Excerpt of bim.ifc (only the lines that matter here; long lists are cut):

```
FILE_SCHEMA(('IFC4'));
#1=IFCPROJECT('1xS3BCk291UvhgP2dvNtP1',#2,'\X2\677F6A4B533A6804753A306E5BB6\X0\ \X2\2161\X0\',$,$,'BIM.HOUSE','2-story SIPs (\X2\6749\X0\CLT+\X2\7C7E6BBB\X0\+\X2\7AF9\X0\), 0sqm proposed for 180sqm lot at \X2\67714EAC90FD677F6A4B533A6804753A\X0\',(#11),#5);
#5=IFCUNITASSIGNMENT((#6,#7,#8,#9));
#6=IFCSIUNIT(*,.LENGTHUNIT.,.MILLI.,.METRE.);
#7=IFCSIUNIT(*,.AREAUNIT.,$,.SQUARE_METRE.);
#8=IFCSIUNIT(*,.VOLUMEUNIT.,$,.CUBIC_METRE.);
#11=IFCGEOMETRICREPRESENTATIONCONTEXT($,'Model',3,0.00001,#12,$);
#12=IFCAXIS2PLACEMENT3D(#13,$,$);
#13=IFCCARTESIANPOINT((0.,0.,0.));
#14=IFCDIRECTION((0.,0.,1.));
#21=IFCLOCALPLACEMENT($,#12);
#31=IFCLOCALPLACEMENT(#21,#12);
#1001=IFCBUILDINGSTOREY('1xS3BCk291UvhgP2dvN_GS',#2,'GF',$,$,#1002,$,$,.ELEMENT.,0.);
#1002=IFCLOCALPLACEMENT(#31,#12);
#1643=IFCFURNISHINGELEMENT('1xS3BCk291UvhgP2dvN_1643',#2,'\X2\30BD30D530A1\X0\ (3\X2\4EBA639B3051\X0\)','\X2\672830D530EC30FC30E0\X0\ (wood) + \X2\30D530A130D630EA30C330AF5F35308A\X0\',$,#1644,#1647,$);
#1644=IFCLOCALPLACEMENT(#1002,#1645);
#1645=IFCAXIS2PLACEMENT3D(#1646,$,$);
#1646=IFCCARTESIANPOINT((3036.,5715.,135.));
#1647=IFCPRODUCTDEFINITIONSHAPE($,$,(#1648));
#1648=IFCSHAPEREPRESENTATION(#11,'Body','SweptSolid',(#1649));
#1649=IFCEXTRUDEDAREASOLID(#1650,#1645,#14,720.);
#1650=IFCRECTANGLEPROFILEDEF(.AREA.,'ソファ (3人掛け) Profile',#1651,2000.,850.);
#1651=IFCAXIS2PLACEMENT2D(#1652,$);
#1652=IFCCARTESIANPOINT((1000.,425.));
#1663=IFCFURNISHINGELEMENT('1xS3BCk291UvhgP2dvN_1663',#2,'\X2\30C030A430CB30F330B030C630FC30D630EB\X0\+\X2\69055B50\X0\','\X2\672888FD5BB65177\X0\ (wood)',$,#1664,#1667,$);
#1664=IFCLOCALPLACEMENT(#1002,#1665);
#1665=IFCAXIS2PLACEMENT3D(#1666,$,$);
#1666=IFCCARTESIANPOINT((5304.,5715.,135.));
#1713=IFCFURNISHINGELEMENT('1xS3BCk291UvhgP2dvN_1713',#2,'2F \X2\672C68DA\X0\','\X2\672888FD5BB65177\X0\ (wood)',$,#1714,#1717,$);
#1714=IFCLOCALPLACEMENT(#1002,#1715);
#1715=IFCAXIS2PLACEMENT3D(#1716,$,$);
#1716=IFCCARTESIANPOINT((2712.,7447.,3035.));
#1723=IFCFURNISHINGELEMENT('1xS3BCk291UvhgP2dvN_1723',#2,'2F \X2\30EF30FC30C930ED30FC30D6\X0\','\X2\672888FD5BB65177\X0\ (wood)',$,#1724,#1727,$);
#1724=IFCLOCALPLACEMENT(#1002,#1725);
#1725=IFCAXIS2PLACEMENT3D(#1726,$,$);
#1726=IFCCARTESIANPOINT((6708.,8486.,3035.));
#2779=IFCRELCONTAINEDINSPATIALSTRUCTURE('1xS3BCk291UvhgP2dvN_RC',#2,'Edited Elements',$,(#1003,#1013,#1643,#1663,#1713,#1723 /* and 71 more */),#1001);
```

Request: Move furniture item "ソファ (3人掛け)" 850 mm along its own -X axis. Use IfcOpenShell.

```python
import ifcopenshell
import ifcopenshell.api.geometry
import ifcopenshell.util.placement

model = ifcopenshell.open("bim.ifc")

item = model.by_guid("1xS3BCk291UvhgP2dvN_1643")
matrix = ifcopenshell.util.placement.get_local_placement(item.ObjectPlacement)
matrix[:3, 3] -= matrix[:3, 0] * 850.0
ifcopenshell.api.geometry.edit_object_placement(model, product=item, matrix=matrix, is_si=False)

print(ifcopenshell.util.placement.get_local_placement(item.ObjectPlacement).round(3) + 0.0)

model.write("bim-out.ifc")
```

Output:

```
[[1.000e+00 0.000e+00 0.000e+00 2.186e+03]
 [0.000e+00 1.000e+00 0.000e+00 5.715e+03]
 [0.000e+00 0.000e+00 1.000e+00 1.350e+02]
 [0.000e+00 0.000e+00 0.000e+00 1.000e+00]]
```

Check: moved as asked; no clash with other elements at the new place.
